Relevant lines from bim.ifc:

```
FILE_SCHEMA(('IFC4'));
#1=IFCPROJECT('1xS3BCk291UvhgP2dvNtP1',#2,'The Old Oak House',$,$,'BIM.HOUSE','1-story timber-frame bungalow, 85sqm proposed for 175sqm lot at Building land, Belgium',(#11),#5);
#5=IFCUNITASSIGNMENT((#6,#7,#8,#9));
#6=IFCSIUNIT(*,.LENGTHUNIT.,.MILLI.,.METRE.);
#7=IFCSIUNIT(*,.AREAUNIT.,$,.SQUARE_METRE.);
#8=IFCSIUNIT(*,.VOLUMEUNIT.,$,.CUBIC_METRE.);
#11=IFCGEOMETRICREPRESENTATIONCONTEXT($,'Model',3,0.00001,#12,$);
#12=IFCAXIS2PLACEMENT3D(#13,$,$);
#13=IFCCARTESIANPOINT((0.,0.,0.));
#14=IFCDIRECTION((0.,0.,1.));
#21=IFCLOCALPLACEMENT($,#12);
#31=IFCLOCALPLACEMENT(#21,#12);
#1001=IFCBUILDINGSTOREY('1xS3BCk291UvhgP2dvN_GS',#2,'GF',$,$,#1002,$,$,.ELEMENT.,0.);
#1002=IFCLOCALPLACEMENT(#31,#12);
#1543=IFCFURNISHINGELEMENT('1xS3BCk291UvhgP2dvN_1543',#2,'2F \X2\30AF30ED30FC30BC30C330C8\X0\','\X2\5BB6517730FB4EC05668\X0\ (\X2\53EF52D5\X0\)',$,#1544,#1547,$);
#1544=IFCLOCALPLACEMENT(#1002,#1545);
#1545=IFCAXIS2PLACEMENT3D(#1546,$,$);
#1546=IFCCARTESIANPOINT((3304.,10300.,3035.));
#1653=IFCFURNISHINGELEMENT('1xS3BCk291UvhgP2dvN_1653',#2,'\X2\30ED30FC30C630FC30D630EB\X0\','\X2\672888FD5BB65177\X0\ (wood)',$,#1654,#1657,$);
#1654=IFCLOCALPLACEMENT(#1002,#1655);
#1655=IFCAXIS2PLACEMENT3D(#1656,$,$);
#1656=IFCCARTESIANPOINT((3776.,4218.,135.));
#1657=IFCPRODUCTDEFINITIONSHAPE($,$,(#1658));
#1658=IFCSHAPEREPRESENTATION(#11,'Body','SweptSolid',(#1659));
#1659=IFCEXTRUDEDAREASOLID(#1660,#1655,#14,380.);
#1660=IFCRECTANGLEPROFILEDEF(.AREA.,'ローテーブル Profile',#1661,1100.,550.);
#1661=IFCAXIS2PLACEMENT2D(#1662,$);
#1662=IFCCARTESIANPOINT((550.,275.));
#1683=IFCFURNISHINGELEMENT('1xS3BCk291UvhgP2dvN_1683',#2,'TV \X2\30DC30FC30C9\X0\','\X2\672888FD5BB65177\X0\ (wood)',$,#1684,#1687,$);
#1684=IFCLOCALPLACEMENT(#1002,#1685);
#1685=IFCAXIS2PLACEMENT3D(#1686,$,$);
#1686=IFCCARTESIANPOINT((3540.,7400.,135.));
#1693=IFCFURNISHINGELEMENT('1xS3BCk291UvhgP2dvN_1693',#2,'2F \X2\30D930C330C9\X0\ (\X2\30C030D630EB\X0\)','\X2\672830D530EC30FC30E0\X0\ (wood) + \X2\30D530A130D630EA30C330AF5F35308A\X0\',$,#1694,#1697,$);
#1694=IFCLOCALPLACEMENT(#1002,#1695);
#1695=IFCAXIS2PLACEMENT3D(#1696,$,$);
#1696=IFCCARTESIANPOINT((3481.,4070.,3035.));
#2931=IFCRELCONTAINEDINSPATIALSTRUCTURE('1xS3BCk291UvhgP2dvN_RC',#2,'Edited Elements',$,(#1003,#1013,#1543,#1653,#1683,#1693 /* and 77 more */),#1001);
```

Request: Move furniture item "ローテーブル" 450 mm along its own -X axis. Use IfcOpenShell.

```python
import ifcopenshell
import ifcopenshell.api.geometry
import ifcopenshell.util.placement
import ifcopenshell.util.unit

model = ifcopenshell.open("bim.ifc")
unit_scale = ifcopenshell.util.unit.calculate_unit_scale(model)

item = model.by_id(1653)
matrix = ifcopenshell.util.placement.get_local_placement(item.ObjectPlacement)
matrix[:3, 3] -= matrix[:3, 0] * 0.45 / unit_scale
ifcopenshell.api.geometry.edit_object_placement(model, product=item, matrix=matrix, is_si=False)

print(ifcopenshell.util.placement.get_local_placement(item.ObjectPlacement).round(3) + 0.0)

model.write("bim-out.ifc")
```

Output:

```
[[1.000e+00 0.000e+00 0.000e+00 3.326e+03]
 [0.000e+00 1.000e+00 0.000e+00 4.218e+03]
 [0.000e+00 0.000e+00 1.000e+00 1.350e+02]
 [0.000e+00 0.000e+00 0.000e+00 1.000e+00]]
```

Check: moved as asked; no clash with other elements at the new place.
